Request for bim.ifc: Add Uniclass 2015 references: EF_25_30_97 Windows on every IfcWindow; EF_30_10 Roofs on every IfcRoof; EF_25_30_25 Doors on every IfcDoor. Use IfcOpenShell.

First a look at what the model holds.

```python
import ifcopenshell

model = ifcopenshell.open("bim.ifc")
print(model.schema)
print("classifications:", [c.Name for c in model.by_type("IfcClassification")])
for ifc_class in ("IfcDoor", "IfcRoof", "IfcStair", "IfcWall", "IfcWindow"):
    print(ifc_class, len(model.by_type(ifc_class)))
```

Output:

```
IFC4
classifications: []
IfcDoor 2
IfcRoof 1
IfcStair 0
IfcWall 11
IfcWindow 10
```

```python
import ifcopenshell
import ifcopenshell.api.classification

model = ifcopenshell.open("bim.ifc")

system = ifcopenshell.api.classification.add_classification(model, classification="Uniclass 2015")

codes = {
    "IfcWindow": ("EF_25_30_97", "Windows"),
    "IfcRoof": ("EF_30_10", "Roofs"),
    "IfcDoor": ("EF_25_30_25", "Doors"),
}
for ifc_class, (code, name) in codes.items():
    products = model.by_type(ifc_class)
    ifcopenshell.api.classification.add_reference(
        model, products=products, classification=system, identification=code, name=name
    )
    print(code, len(products))

model.write("bim-out.ifc")
```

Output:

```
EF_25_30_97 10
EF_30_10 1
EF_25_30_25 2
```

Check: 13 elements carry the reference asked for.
